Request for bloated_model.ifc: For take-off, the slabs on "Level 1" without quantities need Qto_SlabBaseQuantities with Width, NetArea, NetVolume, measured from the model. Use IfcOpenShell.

First a look at what the model holds.

```python
import ifcopenshell
import ifcopenshell.util.element
import ifcopenshell.util.unit

model = ifcopenshell.open("bloated_model.ifc")
print(model.schema)
for unit_type in ("LENGTHUNIT", "AREAUNIT", "VOLUMEUNIT"):
    print(unit_type, ifcopenshell.util.unit.calculate_unit_scale(model, unit_type))
storey = next(s for s in model.by_type("IfcBuildingStorey") if s.Name == "Level 1")
slabs = [e for e in ifcopenshell.util.element.get_decomposition(storey) if e.is_a("IfcSlab")]
for e in sorted(slabs, key=lambda e: e.id()):
    print(e.id(), e.is_a(), e.Name, list(ifcopenshell.util.element.get_psets(e, qtos_only=True)), sep=" | ")
```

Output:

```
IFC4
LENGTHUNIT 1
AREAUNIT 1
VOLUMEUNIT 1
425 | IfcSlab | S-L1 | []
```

```python
import ifcopenshell
import ifcopenshell.api.pset
import ifcopenshell.geom
import ifcopenshell.util.element
import ifcopenshell.util.shape
import ifcopenshell.util.unit

model = ifcopenshell.open("bloated_model.ifc")
unit_scale = ifcopenshell.util.unit.calculate_unit_scale(model)
area_scale = ifcopenshell.util.unit.calculate_unit_scale(model, "AREAUNIT")
volume_scale = ifcopenshell.util.unit.calculate_unit_scale(model, "VOLUMEUNIT")
settings = ifcopenshell.geom.settings()

storey = next(s for s in model.by_type("IfcBuildingStorey") if s.Name == "Level 1")
slabs = [e for e in ifcopenshell.util.element.get_decomposition(storey) if e.is_a("IfcSlab")]

for e in sorted(slabs, key=lambda e: e.id()):
    if ifcopenshell.util.element.get_psets(e, qtos_only=True, should_inherit=False):
        continue
    # Geometry comes back in metres, in the element's own axes.
    shape = ifcopenshell.geom.create_shape(settings, e)
    values = {
        "Width": ifcopenshell.util.shape.get_z(shape.geometry) / unit_scale,
        "NetArea": ifcopenshell.util.shape.get_footprint_area(shape.geometry) / area_scale,
        "NetVolume": ifcopenshell.util.shape.get_volume(shape.geometry) / volume_scale,
    }
    qto = ifcopenshell.api.pset.add_qto(model, product=e, name="Qto_SlabBaseQuantities")
    ifcopenshell.api.pset.edit_qto(model, qto=qto, properties=values)
    print(e.id(), {k: round(v, 3) for k, v in values.items()})

model.write("bloated_model_updated.ifc")
```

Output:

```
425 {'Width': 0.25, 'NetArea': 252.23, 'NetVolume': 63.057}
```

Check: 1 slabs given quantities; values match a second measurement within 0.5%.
